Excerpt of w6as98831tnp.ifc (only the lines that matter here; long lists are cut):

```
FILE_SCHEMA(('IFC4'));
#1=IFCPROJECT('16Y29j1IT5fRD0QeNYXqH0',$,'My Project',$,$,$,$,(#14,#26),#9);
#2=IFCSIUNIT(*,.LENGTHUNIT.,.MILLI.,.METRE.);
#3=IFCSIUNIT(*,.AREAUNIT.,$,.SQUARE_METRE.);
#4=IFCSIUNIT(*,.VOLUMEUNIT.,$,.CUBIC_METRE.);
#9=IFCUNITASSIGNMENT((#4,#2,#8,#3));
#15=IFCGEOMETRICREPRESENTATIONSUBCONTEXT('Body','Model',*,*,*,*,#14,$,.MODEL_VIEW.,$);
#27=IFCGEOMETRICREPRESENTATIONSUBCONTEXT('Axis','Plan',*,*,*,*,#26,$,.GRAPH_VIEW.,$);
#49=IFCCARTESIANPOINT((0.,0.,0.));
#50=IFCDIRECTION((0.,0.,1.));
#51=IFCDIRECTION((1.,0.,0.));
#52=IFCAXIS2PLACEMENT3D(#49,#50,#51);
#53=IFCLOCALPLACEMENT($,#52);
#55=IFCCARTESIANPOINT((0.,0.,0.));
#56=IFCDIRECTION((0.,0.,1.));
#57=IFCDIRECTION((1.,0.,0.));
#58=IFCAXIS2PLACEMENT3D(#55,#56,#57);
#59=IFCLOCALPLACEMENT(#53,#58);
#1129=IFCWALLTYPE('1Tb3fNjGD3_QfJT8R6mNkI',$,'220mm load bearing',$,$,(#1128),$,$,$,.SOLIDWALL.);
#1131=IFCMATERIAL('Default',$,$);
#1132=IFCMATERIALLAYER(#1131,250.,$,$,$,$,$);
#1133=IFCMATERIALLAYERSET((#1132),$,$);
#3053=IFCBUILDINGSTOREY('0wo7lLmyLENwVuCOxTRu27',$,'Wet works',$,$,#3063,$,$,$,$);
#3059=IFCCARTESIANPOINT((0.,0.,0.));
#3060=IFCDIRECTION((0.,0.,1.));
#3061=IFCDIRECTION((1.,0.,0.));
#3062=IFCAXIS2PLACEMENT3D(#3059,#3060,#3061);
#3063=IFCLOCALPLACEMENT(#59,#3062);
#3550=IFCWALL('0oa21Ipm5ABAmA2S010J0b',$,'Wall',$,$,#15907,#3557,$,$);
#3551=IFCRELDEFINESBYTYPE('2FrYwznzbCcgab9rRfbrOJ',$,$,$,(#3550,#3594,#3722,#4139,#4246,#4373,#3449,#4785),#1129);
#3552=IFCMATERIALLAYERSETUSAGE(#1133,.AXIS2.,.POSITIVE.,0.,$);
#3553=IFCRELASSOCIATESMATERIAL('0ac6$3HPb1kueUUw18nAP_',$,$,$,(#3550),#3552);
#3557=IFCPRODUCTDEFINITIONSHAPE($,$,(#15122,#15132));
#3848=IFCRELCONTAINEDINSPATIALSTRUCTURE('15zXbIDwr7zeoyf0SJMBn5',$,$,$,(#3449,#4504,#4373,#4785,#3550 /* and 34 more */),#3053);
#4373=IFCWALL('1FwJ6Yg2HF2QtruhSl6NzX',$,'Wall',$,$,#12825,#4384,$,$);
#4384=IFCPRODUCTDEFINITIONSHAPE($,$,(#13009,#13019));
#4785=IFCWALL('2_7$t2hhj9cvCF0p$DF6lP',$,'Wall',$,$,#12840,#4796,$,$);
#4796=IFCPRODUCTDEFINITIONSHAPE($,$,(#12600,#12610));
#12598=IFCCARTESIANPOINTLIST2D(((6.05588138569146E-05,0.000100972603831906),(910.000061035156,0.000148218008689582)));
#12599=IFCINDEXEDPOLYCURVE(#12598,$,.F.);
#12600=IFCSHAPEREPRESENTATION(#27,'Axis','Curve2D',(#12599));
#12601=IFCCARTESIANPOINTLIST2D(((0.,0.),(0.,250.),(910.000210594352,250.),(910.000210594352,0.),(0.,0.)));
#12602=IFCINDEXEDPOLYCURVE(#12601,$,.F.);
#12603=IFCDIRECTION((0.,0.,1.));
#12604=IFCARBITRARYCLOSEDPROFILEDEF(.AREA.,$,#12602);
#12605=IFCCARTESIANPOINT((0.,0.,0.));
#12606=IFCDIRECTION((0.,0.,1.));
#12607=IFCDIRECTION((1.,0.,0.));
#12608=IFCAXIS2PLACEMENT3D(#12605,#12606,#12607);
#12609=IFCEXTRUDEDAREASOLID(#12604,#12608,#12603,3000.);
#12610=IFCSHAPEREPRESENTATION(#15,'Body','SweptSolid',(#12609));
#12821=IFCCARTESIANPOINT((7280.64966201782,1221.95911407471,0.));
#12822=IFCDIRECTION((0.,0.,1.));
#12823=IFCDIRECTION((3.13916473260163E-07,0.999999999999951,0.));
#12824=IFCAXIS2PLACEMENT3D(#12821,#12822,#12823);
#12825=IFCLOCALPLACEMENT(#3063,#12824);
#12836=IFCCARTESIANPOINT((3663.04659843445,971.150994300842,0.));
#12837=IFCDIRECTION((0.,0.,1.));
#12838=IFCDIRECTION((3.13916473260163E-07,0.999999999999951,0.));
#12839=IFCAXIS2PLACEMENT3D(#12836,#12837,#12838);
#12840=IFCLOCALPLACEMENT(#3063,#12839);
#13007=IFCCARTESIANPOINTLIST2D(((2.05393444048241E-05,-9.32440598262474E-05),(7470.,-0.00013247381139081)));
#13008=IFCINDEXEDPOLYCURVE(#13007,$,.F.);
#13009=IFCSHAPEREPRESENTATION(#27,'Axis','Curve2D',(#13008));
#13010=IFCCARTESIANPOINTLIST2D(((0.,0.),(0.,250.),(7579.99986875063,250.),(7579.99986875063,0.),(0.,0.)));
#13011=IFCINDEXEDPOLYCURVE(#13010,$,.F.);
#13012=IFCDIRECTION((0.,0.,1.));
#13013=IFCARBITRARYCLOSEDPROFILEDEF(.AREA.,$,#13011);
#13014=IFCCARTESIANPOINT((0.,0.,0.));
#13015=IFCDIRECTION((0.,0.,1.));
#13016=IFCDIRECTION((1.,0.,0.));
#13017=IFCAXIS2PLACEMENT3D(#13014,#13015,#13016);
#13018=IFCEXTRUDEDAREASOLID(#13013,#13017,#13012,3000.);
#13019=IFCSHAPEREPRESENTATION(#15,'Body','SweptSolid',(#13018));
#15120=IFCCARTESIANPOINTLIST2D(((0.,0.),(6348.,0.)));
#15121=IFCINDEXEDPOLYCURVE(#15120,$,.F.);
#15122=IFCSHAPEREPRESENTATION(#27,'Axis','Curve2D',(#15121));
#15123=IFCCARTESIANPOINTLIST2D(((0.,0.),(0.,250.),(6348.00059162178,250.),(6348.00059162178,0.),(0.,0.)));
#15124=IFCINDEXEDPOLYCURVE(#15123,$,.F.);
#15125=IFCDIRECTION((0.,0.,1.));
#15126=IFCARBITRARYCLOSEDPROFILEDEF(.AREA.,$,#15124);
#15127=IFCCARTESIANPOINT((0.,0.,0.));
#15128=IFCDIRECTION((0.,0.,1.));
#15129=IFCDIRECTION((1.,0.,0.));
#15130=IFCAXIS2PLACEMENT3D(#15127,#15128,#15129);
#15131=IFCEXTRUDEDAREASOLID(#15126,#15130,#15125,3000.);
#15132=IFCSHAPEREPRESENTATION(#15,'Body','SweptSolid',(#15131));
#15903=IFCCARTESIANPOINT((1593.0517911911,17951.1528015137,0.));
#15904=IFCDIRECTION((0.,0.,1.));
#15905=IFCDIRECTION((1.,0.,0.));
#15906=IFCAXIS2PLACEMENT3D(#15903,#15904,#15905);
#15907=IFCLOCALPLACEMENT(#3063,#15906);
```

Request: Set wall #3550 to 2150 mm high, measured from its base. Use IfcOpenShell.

```python
import ifcopenshell
import ifcopenshell.geom
import ifcopenshell.util.representation
import ifcopenshell.util.shape
import ifcopenshell.util.unit

model = ifcopenshell.open("w6as98831tnp.ifc")
unit_scale = ifcopenshell.util.unit.calculate_unit_scale(model)
settings = ifcopenshell.geom.settings()


def volume(element):
    """Net volume in cubic metres, openings subtracted."""
    shape = ifcopenshell.geom.create_shape(settings, element)
    return ifcopenshell.util.shape.get_volume(shape.geometry)


wall = model.by_guid("0oa21Ipm5ABAmA2S010J0b")
before = volume(wall)

body = ifcopenshell.util.representation.get_representation(wall, "Model", "Body")
solid = body.Items[0]
old_height = solid.Depth
solid.Depth = 2.15 / unit_scale
after = volume(wall)

print(f"height {old_height:g} -> {solid.Depth:g}, volume {before:.3f} -> {after:.3f} m3")

model.write("w6as98831tnp_rev.ifc")
```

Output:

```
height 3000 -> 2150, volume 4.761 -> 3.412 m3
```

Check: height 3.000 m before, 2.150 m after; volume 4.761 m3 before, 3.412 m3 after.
